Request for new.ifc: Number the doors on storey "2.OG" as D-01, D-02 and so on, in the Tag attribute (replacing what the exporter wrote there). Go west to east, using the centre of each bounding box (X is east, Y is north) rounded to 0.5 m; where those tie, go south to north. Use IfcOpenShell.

First a look at what the model holds.

```python
import ifcopenshell
import ifcopenshell.util.element
import ifcopenshell.util.placement

model = ifcopenshell.open("new.ifc")
print(model.schema)
storey = next(s for s in model.by_type("IfcBuildingStorey") if s.Name == "2.OG")
doors = [e for e in ifcopenshell.util.element.get_decomposition(storey) if e.is_a("IfcDoor")]
for e in sorted(doors, key=lambda e: e.id()):
    origin = ifcopenshell.util.placement.get_local_placement(e.ObjectPlacement)[:3, 3]
    print(e.id(), e.Tag, e.Name, origin.round(2) + 0.0, sep=" | ")
```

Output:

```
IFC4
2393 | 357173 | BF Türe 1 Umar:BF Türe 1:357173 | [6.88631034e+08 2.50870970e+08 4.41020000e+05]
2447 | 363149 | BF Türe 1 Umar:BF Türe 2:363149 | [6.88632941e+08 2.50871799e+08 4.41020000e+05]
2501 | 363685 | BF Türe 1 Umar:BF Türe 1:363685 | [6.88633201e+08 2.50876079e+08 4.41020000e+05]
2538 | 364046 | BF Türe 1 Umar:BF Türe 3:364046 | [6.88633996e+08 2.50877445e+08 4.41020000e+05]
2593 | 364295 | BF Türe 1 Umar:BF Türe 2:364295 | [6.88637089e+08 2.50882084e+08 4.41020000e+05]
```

```python
import ifcopenshell
import ifcopenshell.geom
import ifcopenshell.util.element
import ifcopenshell.util.shape

model = ifcopenshell.open("new.ifc")
settings = ifcopenshell.geom.settings()
settings.set("use-world-coords", True)


def centre(element):
    shape = ifcopenshell.geom.create_shape(settings, element)
    return ifcopenshell.util.shape.get_bbox_centroid(shape.geometry)


storey = next(s for s in model.by_type("IfcBuildingStorey") if s.Name == "2.OG")
doors = [e for e in ifcopenshell.util.element.get_decomposition(storey) if e.is_a("IfcDoor")]

# Insertion points can sit at a corner or the storey origin, so sort by the geometry (in metres).
centres = {e: centre(e) for e in doors}
doors.sort(key=lambda e: (round(centres[e][0] / 0.5), centres[e][1]))

for i, e in enumerate(doors, start=1):
    number = f"D-{i:02d}"
    e.Tag = number
    print(e.id(), number)

model.write("new_v2.ifc")
```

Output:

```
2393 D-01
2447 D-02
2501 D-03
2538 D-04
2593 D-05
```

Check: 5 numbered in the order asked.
